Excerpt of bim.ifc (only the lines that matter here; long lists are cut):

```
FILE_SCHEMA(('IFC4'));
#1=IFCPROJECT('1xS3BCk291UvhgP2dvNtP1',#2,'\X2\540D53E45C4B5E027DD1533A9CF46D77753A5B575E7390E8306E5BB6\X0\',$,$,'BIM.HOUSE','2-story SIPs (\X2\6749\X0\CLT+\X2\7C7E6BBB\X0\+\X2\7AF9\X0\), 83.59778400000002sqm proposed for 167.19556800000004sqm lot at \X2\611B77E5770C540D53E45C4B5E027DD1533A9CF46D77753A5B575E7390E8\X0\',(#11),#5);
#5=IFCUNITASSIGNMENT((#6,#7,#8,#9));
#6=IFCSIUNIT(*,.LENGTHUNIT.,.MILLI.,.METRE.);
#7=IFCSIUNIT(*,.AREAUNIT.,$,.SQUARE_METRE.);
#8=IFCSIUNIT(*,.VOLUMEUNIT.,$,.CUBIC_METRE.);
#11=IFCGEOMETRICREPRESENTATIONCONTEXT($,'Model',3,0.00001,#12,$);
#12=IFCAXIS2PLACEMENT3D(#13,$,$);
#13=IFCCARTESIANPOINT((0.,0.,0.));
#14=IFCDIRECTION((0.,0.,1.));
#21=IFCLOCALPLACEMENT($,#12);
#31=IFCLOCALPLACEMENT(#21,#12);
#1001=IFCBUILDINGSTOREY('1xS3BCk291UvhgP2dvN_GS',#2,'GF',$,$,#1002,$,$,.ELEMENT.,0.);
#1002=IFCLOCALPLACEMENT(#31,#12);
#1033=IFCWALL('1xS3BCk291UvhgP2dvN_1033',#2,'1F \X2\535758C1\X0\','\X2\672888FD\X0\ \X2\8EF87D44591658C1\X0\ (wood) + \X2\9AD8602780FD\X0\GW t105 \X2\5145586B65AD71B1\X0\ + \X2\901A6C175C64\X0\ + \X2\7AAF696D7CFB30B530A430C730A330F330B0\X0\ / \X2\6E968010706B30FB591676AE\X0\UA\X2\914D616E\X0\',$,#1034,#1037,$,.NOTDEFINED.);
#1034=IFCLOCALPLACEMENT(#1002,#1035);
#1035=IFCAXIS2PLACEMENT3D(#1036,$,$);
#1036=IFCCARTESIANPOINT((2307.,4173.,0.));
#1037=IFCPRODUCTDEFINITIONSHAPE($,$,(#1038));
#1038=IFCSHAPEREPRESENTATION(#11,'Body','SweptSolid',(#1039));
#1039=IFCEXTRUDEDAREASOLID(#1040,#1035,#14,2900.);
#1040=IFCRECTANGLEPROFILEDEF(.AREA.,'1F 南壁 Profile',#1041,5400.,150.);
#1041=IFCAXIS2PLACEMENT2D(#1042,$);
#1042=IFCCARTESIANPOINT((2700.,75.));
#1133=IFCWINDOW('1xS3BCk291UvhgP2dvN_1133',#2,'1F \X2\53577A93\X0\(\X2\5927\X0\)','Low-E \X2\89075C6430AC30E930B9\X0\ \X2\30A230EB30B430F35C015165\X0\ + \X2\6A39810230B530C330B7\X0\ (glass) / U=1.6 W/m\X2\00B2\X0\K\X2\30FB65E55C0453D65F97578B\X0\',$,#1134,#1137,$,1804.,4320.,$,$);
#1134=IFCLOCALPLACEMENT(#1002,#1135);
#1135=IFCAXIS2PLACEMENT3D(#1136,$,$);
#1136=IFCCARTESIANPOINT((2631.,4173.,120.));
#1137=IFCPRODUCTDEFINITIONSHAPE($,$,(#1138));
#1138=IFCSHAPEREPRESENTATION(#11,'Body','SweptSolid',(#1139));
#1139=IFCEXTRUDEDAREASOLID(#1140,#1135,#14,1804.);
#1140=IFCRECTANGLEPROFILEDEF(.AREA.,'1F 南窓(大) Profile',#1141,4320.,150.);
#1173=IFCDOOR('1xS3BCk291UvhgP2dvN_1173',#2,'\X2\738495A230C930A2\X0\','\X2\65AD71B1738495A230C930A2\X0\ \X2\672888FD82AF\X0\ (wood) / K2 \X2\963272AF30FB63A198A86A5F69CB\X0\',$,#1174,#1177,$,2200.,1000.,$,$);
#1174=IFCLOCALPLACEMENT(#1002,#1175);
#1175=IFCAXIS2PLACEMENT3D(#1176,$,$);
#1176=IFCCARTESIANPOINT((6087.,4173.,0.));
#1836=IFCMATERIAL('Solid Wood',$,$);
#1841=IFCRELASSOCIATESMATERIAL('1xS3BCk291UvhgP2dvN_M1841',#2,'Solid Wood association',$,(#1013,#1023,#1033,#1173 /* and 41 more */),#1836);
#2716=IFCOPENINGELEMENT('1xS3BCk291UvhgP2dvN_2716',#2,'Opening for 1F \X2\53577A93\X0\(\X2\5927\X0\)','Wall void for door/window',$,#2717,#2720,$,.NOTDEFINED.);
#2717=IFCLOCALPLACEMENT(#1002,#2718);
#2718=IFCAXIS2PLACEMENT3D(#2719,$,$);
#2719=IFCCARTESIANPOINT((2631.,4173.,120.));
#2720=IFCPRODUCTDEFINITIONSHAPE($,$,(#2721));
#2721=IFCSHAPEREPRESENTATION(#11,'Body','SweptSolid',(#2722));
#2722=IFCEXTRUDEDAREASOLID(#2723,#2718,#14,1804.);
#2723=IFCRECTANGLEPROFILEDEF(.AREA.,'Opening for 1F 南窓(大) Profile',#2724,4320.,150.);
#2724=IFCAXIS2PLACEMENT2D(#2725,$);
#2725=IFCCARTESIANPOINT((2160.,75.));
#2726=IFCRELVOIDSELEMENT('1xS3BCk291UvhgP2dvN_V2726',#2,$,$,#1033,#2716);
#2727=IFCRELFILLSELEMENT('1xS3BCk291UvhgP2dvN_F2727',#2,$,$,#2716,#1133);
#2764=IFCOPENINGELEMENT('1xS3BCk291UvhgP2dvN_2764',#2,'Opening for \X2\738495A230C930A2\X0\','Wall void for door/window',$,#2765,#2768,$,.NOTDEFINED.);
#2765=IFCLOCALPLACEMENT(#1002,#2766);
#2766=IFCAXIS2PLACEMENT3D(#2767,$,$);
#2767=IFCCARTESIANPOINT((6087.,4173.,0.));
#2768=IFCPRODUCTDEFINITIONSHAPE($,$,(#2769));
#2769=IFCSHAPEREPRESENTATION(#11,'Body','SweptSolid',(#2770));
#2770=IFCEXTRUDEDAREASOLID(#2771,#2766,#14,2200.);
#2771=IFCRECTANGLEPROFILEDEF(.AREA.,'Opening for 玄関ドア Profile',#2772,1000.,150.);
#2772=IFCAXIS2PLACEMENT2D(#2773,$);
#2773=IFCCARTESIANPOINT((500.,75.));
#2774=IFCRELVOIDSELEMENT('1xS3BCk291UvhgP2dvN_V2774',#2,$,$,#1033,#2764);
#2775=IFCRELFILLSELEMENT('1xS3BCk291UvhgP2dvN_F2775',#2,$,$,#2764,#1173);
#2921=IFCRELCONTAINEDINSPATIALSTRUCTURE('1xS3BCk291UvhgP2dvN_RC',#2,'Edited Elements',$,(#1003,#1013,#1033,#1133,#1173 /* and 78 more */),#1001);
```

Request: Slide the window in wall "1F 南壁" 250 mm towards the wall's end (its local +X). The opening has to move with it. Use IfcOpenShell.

```python
import ifcopenshell
import ifcopenshell.api.geometry
import ifcopenshell.util.placement
import ifcopenshell.util.unit

model = ifcopenshell.open("bim.ifc")
unit_scale = ifcopenshell.util.unit.calculate_unit_scale(model)

window = model.by_guid("1xS3BCk291UvhgP2dvN_1133")
opening = window.FillsVoids[0].RelatingOpeningElement
wall = opening.VoidsElements[0].RelatingBuildingElement

wall_matrix = ifcopenshell.util.placement.get_local_placement(wall.ObjectPlacement)
shift = wall_matrix[:3, 0] * 0.25 / unit_scale
before = ifcopenshell.util.placement.get_local_placement(window.ObjectPlacement)[:3, 3].copy()

# The window is not placed relative to its opening, so move both.
for product in (opening, window):
    matrix = ifcopenshell.util.placement.get_local_placement(product.ObjectPlacement)
    matrix[:3, 3] += shift
    ifcopenshell.api.geometry.edit_object_placement(model, product=product, matrix=matrix, is_si=False)

after = ifcopenshell.util.placement.get_local_placement(window.ObjectPlacement)[:3, 3]
print("window moved by", (after - before).round(3) + 0.0)

model.write("bim_edited.ifc")
```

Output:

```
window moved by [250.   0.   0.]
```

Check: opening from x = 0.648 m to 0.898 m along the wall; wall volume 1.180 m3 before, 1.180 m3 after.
